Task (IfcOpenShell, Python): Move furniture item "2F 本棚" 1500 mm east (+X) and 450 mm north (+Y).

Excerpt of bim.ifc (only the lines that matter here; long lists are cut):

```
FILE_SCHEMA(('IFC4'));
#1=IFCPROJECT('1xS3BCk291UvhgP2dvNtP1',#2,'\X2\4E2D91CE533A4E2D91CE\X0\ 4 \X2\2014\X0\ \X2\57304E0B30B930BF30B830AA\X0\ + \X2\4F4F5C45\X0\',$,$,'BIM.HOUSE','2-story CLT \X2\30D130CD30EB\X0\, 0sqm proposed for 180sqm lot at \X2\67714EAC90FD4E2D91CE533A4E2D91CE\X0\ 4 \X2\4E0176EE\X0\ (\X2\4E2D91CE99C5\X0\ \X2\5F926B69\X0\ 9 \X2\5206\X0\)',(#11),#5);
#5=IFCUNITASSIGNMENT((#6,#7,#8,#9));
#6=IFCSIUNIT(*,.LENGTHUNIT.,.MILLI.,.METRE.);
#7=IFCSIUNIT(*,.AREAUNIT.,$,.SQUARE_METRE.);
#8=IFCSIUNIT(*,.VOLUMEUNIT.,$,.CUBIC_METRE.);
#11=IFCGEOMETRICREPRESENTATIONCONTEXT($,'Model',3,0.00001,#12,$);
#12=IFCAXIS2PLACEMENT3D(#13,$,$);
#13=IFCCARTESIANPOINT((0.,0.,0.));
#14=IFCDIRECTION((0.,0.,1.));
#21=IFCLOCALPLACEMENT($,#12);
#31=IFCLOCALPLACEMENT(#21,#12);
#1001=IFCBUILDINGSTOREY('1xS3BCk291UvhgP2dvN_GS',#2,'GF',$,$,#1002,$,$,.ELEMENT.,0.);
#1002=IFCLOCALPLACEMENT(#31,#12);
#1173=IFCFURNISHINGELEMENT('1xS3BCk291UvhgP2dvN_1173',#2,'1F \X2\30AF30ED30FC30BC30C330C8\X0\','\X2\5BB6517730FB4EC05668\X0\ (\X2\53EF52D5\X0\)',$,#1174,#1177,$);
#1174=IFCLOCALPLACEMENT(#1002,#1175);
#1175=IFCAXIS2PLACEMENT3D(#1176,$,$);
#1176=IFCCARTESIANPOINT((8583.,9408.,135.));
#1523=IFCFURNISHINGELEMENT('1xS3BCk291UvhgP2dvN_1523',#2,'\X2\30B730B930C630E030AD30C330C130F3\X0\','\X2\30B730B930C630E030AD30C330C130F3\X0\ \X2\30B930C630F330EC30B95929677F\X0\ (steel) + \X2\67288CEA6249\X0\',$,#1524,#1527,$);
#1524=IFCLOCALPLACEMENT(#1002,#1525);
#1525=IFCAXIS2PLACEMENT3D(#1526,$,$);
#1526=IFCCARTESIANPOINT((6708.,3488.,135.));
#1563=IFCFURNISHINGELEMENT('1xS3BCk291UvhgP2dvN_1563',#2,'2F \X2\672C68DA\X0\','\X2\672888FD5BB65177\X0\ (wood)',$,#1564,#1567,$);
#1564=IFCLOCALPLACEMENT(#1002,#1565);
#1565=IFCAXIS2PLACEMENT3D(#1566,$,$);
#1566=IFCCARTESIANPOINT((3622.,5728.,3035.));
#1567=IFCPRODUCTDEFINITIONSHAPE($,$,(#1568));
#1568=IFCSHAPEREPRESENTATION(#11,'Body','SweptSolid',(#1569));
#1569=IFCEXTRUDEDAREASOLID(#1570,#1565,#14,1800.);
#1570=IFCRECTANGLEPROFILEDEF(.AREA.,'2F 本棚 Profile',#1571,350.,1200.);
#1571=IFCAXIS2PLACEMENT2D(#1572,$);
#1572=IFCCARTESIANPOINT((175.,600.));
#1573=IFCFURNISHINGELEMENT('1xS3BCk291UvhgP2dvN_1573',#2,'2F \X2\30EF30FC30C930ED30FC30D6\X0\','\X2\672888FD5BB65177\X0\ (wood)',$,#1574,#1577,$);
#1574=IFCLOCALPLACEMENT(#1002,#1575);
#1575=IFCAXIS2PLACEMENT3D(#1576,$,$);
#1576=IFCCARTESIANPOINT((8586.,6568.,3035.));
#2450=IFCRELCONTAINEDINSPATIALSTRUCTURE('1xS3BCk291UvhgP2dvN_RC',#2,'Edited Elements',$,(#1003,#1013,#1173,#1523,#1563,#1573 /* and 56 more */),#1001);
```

```python
import ifcopenshell
import ifcopenshell.api.geometry
import ifcopenshell.util.placement

model = ifcopenshell.open("bim.ifc")

item = model.by_id(1563)
matrix = ifcopenshell.util.placement.get_local_placement(item.ObjectPlacement)
matrix[0, 3] += 1500.0
matrix[1, 3] += 450.0
ifcopenshell.api.geometry.edit_object_placement(model, product=item, matrix=matrix, is_si=False)

print(ifcopenshell.util.placement.get_local_placement(item.ObjectPlacement).round(3) + 0.0)

model.write("bim_rev.ifc")
```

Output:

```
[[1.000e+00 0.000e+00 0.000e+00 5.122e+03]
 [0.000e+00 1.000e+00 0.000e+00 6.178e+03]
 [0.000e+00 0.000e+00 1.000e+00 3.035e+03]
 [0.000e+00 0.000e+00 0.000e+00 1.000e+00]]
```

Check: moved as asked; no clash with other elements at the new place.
